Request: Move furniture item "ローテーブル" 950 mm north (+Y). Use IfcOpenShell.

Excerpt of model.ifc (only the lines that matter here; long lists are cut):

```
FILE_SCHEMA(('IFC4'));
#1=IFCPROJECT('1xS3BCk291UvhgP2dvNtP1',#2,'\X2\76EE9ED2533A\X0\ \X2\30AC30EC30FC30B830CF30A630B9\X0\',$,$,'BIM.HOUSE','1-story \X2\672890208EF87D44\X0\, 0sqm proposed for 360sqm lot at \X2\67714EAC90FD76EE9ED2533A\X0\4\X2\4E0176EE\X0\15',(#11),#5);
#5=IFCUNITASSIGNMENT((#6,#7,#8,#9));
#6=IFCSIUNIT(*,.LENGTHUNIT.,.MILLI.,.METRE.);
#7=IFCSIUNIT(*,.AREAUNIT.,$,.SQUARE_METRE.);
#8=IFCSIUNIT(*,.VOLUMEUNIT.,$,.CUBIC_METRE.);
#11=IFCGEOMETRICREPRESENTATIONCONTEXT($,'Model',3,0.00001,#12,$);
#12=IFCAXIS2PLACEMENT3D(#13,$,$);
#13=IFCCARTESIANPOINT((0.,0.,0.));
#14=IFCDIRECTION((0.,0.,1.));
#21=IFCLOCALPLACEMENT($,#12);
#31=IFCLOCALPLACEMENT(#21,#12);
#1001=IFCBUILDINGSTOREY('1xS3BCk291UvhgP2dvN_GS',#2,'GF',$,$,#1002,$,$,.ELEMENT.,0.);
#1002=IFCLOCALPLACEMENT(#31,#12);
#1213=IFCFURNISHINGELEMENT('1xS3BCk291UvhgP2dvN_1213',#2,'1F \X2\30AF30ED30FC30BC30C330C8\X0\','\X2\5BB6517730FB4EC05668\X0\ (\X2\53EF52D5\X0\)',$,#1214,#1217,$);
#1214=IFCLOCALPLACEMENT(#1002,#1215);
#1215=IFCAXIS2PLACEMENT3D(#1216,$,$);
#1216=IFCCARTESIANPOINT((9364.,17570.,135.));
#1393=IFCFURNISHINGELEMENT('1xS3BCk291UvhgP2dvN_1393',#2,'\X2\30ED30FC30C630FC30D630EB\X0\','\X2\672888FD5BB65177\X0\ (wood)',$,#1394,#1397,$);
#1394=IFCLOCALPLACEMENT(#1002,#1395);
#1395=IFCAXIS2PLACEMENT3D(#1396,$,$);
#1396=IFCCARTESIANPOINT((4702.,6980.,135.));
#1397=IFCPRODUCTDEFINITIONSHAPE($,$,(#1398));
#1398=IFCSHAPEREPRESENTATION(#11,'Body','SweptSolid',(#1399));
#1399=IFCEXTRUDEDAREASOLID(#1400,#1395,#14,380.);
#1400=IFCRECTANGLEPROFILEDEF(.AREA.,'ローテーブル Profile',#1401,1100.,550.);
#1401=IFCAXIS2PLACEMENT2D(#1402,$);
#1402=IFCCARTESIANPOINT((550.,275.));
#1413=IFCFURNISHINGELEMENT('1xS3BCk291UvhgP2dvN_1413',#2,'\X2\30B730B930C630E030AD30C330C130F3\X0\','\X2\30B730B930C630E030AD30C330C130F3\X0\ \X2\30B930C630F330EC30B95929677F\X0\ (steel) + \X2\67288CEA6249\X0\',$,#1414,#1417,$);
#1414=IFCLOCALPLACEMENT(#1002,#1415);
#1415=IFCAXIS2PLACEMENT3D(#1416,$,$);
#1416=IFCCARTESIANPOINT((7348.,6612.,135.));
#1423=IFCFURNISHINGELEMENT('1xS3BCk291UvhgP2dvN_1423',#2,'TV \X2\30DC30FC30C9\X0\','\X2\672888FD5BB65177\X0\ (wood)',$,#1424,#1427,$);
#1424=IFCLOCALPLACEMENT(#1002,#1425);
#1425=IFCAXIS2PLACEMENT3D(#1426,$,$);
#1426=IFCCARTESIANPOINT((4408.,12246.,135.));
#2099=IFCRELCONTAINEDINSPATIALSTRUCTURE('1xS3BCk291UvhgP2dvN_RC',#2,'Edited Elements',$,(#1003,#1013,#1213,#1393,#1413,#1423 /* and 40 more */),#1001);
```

```python
import ifcopenshell
import ifcopenshell.api.geometry
import ifcopenshell.util.placement

model = ifcopenshell.open("model.ifc")

item = model.by_id(1393)
matrix = ifcopenshell.util.placement.get_local_placement(item.ObjectPlacement)
matrix[1, 3] += 950.0
ifcopenshell.api.geometry.edit_object_placement(model, product=item, matrix=matrix, is_si=False)

print(ifcopenshell.util.placement.get_local_placement(item.ObjectPlacement).round(3) + 0.0)

model.write("model-out.ifc")
```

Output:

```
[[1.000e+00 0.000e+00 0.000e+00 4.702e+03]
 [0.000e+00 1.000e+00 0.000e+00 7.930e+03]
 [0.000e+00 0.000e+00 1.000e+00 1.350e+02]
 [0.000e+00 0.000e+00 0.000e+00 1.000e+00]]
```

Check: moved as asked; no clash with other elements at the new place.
